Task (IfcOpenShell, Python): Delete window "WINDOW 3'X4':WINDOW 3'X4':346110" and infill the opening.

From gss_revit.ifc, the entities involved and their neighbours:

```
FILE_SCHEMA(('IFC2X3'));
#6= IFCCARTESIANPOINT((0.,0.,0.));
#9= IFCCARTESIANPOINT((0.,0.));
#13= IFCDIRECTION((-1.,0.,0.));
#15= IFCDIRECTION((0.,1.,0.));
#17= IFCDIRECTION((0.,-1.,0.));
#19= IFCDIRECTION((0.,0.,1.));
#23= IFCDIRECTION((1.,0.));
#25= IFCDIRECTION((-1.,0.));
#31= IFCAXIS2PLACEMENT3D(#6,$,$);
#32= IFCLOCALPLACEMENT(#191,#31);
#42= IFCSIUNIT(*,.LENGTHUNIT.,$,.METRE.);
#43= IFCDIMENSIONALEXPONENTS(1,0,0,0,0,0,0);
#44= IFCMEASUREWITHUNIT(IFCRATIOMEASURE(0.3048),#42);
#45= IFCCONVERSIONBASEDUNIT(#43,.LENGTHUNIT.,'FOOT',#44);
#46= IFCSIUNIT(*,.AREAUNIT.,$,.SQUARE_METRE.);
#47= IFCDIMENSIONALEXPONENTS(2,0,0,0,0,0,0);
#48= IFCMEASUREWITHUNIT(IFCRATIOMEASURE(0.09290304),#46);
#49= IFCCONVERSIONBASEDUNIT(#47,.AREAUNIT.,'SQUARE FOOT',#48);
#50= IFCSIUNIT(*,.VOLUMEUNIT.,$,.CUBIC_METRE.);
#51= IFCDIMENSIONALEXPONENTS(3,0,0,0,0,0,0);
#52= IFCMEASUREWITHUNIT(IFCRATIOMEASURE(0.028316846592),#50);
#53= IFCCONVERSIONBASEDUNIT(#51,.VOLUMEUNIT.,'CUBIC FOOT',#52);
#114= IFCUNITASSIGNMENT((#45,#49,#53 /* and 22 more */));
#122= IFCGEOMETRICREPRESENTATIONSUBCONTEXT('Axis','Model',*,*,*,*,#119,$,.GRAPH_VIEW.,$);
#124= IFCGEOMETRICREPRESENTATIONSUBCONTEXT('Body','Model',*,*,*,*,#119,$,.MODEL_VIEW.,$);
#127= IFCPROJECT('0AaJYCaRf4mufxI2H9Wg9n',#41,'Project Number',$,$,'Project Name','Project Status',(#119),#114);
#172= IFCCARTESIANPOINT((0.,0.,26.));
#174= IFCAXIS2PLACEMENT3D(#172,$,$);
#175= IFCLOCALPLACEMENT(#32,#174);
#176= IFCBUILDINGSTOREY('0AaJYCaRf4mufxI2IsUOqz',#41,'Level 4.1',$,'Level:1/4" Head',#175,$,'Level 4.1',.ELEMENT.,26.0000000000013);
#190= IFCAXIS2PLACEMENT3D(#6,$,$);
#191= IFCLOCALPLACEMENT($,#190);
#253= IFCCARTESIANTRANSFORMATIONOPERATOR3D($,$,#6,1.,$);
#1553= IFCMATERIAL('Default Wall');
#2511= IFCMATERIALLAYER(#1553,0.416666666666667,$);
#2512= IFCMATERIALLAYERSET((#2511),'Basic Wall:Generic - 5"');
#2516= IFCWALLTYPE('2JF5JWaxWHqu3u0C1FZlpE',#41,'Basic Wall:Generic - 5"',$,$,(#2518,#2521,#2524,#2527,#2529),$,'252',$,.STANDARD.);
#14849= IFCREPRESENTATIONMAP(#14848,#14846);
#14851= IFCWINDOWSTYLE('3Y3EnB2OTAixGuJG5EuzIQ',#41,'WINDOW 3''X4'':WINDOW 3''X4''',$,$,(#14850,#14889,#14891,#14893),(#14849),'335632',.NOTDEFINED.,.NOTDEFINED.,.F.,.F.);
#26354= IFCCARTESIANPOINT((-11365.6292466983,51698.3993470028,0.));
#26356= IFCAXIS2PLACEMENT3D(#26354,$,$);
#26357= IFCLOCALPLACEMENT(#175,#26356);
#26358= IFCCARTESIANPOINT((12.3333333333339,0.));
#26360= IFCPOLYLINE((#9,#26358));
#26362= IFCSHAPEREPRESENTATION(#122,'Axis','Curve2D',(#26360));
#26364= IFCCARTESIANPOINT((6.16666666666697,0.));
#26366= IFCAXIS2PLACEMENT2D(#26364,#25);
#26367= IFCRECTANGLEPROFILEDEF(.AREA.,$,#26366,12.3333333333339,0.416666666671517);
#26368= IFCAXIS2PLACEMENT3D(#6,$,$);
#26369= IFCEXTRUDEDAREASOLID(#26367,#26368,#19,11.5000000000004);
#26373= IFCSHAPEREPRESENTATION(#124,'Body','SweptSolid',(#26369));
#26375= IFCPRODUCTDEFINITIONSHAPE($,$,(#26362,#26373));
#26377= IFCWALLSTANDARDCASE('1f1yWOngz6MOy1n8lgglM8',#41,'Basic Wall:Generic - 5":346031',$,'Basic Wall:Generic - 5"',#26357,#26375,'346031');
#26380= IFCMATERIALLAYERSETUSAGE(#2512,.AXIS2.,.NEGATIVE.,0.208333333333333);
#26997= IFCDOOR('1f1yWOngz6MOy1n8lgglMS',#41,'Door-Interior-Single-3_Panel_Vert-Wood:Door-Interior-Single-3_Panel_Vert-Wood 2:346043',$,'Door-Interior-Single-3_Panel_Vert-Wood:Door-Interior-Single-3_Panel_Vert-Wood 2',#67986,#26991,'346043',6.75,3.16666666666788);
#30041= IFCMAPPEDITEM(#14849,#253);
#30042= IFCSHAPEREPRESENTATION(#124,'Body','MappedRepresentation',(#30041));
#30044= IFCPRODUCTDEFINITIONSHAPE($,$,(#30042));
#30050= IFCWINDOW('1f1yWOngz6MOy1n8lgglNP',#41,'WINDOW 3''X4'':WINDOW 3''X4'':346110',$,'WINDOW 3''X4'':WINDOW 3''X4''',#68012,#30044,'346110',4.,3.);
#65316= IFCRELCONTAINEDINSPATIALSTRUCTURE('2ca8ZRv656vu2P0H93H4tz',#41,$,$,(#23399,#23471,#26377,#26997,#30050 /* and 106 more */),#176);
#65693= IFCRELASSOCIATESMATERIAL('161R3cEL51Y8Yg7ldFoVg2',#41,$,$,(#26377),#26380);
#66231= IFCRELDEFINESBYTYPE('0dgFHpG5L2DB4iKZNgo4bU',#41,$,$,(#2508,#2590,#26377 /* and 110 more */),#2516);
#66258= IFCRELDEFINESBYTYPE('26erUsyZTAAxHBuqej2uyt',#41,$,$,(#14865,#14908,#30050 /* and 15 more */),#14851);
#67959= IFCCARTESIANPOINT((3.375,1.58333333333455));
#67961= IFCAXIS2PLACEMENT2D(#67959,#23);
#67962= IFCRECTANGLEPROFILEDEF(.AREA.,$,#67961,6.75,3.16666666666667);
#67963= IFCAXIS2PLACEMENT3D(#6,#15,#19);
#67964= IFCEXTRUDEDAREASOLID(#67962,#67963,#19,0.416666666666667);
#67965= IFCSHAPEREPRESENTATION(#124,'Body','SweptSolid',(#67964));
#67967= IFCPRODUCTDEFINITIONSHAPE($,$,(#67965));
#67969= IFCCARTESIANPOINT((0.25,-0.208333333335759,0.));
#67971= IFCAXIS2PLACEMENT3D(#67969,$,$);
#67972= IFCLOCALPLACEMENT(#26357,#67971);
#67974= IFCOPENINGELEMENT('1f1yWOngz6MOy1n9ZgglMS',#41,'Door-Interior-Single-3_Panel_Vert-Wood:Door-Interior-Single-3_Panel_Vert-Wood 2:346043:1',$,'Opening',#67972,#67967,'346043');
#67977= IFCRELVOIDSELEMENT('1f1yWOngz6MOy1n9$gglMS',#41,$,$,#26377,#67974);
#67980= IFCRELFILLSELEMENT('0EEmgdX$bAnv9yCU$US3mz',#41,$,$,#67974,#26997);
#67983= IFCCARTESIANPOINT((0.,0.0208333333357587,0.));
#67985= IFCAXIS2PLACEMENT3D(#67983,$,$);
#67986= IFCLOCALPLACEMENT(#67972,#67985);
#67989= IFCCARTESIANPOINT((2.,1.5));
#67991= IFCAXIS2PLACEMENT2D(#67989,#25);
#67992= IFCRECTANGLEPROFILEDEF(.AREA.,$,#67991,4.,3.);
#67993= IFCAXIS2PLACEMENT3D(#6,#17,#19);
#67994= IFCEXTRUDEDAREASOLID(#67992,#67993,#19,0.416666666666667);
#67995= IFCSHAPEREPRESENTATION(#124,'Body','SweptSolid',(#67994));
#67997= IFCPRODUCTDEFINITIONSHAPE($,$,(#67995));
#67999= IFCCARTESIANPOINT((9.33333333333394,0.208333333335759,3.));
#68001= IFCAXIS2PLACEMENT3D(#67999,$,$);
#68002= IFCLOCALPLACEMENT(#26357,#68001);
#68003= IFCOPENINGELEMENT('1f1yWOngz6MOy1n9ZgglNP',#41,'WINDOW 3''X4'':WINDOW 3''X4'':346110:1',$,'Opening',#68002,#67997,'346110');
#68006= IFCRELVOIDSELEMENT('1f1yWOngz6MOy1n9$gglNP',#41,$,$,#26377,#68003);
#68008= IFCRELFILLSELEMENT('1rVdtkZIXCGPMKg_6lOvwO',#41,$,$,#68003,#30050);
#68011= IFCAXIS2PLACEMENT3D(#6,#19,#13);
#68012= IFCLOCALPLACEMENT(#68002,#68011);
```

```python
import ifcopenshell
import ifcopenshell.api.feature
import ifcopenshell.api.root
import ifcopenshell.geom
import ifcopenshell.util.shape

model = ifcopenshell.open("gss_revit.ifc")
settings = ifcopenshell.geom.settings()


def volume(element):
    """Net volume in cubic metres, openings subtracted."""
    shape = ifcopenshell.geom.create_shape(settings, element)
    return ifcopenshell.util.shape.get_volume(shape.geometry)


window = model.by_id(30050)
opening = window.FillsVoids[0].RelatingOpeningElement
wall = opening.VoidsElements[0].RelatingBuildingElement
before = volume(wall)

ifcopenshell.api.root.remove_product(model, product=window)
ifcopenshell.api.feature.remove_feature(model, feature=opening)

after = volume(wall)

print(f"wall volume {before:.3f} -> {after:.3f} m3")

model.write("gss_revit_v2.ifc")
```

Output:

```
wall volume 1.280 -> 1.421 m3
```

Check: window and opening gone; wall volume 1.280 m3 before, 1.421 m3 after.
